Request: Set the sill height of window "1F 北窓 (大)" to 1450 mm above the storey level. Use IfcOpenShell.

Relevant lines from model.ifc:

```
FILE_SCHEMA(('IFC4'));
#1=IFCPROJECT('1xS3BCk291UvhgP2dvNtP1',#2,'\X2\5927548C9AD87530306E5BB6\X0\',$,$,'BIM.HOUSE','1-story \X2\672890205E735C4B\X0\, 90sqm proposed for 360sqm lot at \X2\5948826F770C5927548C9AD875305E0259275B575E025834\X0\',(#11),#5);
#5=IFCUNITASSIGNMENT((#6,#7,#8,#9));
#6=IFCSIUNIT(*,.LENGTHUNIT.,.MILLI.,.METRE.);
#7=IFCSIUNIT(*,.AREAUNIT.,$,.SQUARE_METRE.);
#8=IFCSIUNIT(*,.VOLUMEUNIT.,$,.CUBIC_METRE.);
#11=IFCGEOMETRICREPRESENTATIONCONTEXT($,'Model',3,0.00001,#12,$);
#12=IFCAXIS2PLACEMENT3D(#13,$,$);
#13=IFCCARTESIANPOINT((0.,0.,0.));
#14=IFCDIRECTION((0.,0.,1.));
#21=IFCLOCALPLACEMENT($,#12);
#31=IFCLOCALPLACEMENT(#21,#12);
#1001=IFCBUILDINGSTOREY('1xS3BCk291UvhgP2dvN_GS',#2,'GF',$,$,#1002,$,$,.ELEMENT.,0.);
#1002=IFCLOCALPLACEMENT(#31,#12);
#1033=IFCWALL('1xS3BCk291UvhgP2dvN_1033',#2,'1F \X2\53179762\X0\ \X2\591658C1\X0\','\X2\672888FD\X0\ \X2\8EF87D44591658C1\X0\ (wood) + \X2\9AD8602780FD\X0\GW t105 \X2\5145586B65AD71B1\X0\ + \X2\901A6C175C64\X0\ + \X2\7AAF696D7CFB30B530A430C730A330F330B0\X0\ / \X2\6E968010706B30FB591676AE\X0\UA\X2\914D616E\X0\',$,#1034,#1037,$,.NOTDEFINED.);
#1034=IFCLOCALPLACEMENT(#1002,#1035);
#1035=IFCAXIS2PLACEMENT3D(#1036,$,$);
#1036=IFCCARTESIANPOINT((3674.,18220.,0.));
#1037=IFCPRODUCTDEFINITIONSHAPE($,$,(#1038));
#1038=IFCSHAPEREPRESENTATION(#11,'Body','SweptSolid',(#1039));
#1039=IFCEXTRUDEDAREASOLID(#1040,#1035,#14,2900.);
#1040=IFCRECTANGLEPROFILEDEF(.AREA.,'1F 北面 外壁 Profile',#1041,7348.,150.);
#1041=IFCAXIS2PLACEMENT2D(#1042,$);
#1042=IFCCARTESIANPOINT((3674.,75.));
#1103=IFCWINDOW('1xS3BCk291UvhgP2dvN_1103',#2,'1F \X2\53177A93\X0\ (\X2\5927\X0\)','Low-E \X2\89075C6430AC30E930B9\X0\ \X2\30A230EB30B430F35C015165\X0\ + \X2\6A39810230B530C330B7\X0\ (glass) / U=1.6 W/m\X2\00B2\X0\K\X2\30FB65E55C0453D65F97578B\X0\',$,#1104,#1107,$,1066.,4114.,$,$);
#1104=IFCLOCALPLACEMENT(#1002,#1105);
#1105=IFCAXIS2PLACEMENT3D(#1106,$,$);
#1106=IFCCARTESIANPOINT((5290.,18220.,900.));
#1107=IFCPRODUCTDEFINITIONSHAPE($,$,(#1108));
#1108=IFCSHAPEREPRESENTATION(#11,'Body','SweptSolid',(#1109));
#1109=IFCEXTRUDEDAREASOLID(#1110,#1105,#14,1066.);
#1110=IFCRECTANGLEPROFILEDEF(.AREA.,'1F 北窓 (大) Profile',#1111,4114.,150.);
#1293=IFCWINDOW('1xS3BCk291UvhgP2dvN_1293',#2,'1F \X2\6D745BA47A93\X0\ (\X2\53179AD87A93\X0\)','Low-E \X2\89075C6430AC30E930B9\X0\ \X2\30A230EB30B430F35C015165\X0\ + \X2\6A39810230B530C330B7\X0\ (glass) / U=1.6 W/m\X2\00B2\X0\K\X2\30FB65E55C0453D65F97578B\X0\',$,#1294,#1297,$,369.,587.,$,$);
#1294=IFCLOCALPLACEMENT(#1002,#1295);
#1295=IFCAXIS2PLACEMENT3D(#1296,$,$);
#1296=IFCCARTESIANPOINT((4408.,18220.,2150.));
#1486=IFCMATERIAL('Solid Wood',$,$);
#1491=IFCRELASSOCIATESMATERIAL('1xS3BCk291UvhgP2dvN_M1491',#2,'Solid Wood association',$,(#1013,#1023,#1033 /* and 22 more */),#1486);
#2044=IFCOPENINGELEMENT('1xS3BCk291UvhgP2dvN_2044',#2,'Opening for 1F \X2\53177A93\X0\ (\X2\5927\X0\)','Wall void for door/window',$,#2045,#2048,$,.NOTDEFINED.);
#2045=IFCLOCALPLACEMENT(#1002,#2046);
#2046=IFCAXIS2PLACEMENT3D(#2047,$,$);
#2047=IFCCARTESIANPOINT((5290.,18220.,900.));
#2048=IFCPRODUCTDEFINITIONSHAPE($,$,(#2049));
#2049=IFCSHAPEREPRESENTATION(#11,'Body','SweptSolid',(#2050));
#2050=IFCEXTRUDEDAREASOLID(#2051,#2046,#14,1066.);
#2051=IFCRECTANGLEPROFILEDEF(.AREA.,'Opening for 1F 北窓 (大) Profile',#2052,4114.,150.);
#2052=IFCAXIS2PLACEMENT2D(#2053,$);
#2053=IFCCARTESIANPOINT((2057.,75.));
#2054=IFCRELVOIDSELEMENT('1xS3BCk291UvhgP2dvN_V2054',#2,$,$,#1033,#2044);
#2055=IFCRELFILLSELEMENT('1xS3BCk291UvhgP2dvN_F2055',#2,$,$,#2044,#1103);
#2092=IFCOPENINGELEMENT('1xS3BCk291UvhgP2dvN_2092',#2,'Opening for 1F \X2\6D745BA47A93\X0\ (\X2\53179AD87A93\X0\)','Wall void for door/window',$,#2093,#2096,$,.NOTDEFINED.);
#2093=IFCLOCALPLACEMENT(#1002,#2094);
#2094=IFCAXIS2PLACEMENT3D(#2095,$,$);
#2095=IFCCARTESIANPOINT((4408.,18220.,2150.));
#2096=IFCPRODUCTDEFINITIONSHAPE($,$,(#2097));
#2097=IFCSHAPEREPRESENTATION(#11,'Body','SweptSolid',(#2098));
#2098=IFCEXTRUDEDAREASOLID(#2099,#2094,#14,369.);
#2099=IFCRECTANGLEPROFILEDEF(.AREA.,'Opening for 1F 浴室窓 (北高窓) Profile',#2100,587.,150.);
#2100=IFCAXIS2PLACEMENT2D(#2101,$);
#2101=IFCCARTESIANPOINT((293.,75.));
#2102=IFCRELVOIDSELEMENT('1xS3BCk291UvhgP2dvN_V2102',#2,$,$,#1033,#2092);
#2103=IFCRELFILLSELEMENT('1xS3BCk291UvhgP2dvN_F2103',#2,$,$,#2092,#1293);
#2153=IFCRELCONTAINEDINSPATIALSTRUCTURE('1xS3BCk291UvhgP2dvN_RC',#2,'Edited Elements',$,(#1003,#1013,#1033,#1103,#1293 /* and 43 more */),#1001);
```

```python
import numpy as np
import ifcopenshell
import ifcopenshell.api.geometry
import ifcopenshell.geom
import ifcopenshell.util.element
import ifcopenshell.util.placement
import ifcopenshell.util.shape
import ifcopenshell.util.unit

model = ifcopenshell.open("model.ifc")
unit_scale = ifcopenshell.util.unit.calculate_unit_scale(model)

window = model.by_guid("1xS3BCk291UvhgP2dvN_1103")
opening = window.FillsVoids[0].RelatingOpeningElement
storey = ifcopenshell.util.element.get_container(window, ifc_class="IfcBuildingStorey")
level = ifcopenshell.util.placement.get_local_placement(storey.ObjectPlacement)[2, 3]

# The opening's origin need not be at the sill, so measure its lowest point.
shape = ifcopenshell.geom.create_shape(ifcopenshell.geom.settings(), opening)
bottom = ifcopenshell.util.shape.get_shape_bottom_elevation(shape, shape.geometry) / unit_scale
dz = level + 1450.0 - bottom

shift = np.array([0.0, 0.0, dz])
# The window is not placed relative to its opening, so move both.
for product in (opening, window):
    matrix = ifcopenshell.util.placement.get_local_placement(product.ObjectPlacement)
    matrix[:3, 3] += shift
    ifcopenshell.api.geometry.edit_object_placement(model, product=product, matrix=matrix, is_si=False)

print(f"moved by {dz * unit_scale:+.3f} m")

model.write("model_rev.ifc")
```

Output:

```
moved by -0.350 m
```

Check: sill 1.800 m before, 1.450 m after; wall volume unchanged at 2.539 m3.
